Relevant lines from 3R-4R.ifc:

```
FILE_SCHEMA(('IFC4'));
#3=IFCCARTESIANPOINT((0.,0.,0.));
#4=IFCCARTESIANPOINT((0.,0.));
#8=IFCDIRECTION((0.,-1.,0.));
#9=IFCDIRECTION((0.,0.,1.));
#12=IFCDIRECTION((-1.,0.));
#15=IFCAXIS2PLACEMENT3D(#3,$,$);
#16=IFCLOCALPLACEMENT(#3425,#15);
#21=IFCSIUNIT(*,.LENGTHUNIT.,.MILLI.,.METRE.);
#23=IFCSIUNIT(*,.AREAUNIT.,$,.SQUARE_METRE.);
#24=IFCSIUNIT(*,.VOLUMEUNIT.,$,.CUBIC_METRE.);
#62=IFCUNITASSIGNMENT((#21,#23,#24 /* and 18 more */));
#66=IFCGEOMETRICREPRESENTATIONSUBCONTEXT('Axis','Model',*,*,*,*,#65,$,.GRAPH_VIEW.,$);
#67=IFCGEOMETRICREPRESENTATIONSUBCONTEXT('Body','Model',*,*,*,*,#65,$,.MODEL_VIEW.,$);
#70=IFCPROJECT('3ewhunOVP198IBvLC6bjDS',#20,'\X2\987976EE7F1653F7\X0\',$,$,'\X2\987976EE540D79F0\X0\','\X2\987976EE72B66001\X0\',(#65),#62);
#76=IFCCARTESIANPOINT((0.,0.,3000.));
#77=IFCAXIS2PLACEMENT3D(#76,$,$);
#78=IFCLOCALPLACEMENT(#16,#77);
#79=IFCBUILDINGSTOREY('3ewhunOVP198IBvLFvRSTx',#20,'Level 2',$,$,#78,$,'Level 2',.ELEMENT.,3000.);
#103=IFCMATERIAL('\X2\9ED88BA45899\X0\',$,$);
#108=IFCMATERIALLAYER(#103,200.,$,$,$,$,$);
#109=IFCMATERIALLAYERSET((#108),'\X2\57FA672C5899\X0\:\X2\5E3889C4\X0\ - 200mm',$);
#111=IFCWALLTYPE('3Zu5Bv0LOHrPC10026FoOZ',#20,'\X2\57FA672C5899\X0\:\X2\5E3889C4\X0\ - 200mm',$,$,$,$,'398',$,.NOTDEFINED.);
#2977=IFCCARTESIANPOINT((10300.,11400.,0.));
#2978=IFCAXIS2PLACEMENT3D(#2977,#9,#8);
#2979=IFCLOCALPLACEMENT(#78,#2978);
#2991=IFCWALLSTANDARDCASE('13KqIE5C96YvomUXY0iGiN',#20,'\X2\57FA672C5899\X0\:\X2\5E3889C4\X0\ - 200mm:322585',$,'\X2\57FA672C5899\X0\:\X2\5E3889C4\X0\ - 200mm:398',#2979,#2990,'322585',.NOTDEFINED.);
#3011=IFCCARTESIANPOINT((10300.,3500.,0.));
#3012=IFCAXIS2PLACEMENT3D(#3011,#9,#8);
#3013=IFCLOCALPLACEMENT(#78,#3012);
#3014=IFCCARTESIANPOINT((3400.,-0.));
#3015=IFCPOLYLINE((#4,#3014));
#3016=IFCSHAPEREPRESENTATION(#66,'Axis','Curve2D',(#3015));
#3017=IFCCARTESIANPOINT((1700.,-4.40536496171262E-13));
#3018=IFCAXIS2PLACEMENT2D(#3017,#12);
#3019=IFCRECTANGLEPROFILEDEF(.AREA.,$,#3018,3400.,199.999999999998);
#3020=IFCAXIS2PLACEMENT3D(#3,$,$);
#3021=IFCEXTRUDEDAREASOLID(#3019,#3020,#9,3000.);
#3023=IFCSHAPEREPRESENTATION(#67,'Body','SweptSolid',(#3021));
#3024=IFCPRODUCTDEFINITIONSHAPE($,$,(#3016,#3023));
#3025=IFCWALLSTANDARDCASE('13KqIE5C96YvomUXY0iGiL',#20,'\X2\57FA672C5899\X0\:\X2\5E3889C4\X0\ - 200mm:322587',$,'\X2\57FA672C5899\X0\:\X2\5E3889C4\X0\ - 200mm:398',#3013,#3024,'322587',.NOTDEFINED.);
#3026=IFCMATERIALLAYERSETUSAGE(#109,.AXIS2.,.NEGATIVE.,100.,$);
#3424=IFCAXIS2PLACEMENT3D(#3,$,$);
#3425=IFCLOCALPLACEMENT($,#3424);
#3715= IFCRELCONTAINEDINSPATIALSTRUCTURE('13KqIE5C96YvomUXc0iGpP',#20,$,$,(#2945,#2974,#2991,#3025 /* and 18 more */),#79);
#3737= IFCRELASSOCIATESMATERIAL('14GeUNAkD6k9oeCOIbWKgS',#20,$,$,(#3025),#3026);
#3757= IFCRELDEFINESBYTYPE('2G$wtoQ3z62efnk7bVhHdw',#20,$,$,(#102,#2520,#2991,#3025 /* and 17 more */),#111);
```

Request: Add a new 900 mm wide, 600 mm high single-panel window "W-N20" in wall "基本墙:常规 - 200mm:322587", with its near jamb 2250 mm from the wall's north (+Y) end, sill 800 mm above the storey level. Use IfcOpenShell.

```python
import numpy as np
import ifcopenshell
import ifcopenshell.api.feature
import ifcopenshell.api.geometry
import ifcopenshell.api.root
import ifcopenshell.api.spatial
import ifcopenshell.geom
import ifcopenshell.util.element
import ifcopenshell.util.placement
import ifcopenshell.util.representation
import ifcopenshell.util.shape
import ifcopenshell.util.unit

model = ifcopenshell.open("3R-4R.ifc")
unit_scale = ifcopenshell.util.unit.calculate_unit_scale(model)
settings = ifcopenshell.geom.settings()


def volume(element):
    """Net volume in cubic metres, openings subtracted."""
    shape = ifcopenshell.geom.create_shape(settings, element)
    return ifcopenshell.util.shape.get_volume(shape.geometry)


wall = model.by_guid("13KqIE5C96YvomUXY0iGiL")
storey = ifcopenshell.util.element.get_container(wall, ifc_class="IfcBuildingStorey")
context = ifcopenshell.util.representation.get_context(model, "Model", "Body", "MODEL_VIEW")
before = volume(wall)

width, height, from_end, sill = 0.9, 0.6, 2.25, 0.8  # metres

# The wall runs along its own X axis, and the end named is its -X end.
wall_shape = ifcopenshell.geom.create_shape(settings, wall)
x, y, z = ifcopenshell.util.shape.get_vertices(wall_shape.geometry).T
start = x.min() + from_end
face, thickness = float(y.min()), float(y.max() - y.min())
wall_matrix = ifcopenshell.util.placement.get_local_placement(wall.ObjectPlacement)
level = ifcopenshell.util.placement.get_local_placement(storey.ObjectPlacement)[2, 3]


def in_wall(x, y):
    """Placement at x, y metres in the wall's axes, at sill height."""
    matrix = wall_matrix.copy()
    matrix[:, 3] = wall_matrix @ np.array([x / unit_scale, y / unit_scale, 0.0, 1.0])
    matrix[2, 3] = level + sill / unit_scale
    return matrix


# Opening: a box that overshoots both wall faces by 50 mm.
opening = ifcopenshell.api.root.create_entity(model, ifc_class="IfcOpeningElement", predefined_type="OPENING")
box = ifcopenshell.api.geometry.add_wall_representation(
    model, context=context, length=width, height=height, thickness=thickness + 0.1
)
ifcopenshell.api.geometry.assign_representation(model, product=opening, representation=box)
ifcopenshell.api.geometry.edit_object_placement(model, product=opening, matrix=in_wall(start, face - 0.05), is_si=False)
ifcopenshell.api.feature.add_feature(model, feature=opening, element=wall)

window = ifcopenshell.api.root.create_entity(model, ifc_class="IfcWindow", name="W-N20", predefined_type="WINDOW")
window.OverallWidth, window.OverallHeight = width / unit_scale, height / unit_scale
window.PartitioningType = "SINGLE_PANEL"
body = ifcopenshell.api.geometry.add_window_representation(
    model,
    context=context,
    overall_width=window.OverallWidth,
    overall_height=window.OverallHeight,
    partition_type="SINGLE_PANEL",
)
ifcopenshell.api.geometry.assign_representation(model, product=window, representation=body)
ifcopenshell.api.spatial.assign_container(model, products=[window], relating_structure=storey)
ifcopenshell.api.feature.add_filling(model, opening=opening, element=window)

# Centre the window in the wall's thickness.
ifcopenshell.api.geometry.edit_object_placement(model, product=window, matrix=in_wall(start, face), is_si=False)
window_shape = ifcopenshell.geom.create_shape(settings, window)
depth = ifcopenshell.util.shape.get_vertices(window_shape.geometry)[:, 1]
offset = face + thickness / 2 - (depth.min() + depth.max()) / 2
ifcopenshell.api.geometry.edit_object_placement(model, product=window, matrix=in_wall(start, offset), is_si=False)

after = volume(wall)

print(f"wall volume {before:.3f} -> {after:.3f} m3")

model.write("3R-4R-out.ifc")
```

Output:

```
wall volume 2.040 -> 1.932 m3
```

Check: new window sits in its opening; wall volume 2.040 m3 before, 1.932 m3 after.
